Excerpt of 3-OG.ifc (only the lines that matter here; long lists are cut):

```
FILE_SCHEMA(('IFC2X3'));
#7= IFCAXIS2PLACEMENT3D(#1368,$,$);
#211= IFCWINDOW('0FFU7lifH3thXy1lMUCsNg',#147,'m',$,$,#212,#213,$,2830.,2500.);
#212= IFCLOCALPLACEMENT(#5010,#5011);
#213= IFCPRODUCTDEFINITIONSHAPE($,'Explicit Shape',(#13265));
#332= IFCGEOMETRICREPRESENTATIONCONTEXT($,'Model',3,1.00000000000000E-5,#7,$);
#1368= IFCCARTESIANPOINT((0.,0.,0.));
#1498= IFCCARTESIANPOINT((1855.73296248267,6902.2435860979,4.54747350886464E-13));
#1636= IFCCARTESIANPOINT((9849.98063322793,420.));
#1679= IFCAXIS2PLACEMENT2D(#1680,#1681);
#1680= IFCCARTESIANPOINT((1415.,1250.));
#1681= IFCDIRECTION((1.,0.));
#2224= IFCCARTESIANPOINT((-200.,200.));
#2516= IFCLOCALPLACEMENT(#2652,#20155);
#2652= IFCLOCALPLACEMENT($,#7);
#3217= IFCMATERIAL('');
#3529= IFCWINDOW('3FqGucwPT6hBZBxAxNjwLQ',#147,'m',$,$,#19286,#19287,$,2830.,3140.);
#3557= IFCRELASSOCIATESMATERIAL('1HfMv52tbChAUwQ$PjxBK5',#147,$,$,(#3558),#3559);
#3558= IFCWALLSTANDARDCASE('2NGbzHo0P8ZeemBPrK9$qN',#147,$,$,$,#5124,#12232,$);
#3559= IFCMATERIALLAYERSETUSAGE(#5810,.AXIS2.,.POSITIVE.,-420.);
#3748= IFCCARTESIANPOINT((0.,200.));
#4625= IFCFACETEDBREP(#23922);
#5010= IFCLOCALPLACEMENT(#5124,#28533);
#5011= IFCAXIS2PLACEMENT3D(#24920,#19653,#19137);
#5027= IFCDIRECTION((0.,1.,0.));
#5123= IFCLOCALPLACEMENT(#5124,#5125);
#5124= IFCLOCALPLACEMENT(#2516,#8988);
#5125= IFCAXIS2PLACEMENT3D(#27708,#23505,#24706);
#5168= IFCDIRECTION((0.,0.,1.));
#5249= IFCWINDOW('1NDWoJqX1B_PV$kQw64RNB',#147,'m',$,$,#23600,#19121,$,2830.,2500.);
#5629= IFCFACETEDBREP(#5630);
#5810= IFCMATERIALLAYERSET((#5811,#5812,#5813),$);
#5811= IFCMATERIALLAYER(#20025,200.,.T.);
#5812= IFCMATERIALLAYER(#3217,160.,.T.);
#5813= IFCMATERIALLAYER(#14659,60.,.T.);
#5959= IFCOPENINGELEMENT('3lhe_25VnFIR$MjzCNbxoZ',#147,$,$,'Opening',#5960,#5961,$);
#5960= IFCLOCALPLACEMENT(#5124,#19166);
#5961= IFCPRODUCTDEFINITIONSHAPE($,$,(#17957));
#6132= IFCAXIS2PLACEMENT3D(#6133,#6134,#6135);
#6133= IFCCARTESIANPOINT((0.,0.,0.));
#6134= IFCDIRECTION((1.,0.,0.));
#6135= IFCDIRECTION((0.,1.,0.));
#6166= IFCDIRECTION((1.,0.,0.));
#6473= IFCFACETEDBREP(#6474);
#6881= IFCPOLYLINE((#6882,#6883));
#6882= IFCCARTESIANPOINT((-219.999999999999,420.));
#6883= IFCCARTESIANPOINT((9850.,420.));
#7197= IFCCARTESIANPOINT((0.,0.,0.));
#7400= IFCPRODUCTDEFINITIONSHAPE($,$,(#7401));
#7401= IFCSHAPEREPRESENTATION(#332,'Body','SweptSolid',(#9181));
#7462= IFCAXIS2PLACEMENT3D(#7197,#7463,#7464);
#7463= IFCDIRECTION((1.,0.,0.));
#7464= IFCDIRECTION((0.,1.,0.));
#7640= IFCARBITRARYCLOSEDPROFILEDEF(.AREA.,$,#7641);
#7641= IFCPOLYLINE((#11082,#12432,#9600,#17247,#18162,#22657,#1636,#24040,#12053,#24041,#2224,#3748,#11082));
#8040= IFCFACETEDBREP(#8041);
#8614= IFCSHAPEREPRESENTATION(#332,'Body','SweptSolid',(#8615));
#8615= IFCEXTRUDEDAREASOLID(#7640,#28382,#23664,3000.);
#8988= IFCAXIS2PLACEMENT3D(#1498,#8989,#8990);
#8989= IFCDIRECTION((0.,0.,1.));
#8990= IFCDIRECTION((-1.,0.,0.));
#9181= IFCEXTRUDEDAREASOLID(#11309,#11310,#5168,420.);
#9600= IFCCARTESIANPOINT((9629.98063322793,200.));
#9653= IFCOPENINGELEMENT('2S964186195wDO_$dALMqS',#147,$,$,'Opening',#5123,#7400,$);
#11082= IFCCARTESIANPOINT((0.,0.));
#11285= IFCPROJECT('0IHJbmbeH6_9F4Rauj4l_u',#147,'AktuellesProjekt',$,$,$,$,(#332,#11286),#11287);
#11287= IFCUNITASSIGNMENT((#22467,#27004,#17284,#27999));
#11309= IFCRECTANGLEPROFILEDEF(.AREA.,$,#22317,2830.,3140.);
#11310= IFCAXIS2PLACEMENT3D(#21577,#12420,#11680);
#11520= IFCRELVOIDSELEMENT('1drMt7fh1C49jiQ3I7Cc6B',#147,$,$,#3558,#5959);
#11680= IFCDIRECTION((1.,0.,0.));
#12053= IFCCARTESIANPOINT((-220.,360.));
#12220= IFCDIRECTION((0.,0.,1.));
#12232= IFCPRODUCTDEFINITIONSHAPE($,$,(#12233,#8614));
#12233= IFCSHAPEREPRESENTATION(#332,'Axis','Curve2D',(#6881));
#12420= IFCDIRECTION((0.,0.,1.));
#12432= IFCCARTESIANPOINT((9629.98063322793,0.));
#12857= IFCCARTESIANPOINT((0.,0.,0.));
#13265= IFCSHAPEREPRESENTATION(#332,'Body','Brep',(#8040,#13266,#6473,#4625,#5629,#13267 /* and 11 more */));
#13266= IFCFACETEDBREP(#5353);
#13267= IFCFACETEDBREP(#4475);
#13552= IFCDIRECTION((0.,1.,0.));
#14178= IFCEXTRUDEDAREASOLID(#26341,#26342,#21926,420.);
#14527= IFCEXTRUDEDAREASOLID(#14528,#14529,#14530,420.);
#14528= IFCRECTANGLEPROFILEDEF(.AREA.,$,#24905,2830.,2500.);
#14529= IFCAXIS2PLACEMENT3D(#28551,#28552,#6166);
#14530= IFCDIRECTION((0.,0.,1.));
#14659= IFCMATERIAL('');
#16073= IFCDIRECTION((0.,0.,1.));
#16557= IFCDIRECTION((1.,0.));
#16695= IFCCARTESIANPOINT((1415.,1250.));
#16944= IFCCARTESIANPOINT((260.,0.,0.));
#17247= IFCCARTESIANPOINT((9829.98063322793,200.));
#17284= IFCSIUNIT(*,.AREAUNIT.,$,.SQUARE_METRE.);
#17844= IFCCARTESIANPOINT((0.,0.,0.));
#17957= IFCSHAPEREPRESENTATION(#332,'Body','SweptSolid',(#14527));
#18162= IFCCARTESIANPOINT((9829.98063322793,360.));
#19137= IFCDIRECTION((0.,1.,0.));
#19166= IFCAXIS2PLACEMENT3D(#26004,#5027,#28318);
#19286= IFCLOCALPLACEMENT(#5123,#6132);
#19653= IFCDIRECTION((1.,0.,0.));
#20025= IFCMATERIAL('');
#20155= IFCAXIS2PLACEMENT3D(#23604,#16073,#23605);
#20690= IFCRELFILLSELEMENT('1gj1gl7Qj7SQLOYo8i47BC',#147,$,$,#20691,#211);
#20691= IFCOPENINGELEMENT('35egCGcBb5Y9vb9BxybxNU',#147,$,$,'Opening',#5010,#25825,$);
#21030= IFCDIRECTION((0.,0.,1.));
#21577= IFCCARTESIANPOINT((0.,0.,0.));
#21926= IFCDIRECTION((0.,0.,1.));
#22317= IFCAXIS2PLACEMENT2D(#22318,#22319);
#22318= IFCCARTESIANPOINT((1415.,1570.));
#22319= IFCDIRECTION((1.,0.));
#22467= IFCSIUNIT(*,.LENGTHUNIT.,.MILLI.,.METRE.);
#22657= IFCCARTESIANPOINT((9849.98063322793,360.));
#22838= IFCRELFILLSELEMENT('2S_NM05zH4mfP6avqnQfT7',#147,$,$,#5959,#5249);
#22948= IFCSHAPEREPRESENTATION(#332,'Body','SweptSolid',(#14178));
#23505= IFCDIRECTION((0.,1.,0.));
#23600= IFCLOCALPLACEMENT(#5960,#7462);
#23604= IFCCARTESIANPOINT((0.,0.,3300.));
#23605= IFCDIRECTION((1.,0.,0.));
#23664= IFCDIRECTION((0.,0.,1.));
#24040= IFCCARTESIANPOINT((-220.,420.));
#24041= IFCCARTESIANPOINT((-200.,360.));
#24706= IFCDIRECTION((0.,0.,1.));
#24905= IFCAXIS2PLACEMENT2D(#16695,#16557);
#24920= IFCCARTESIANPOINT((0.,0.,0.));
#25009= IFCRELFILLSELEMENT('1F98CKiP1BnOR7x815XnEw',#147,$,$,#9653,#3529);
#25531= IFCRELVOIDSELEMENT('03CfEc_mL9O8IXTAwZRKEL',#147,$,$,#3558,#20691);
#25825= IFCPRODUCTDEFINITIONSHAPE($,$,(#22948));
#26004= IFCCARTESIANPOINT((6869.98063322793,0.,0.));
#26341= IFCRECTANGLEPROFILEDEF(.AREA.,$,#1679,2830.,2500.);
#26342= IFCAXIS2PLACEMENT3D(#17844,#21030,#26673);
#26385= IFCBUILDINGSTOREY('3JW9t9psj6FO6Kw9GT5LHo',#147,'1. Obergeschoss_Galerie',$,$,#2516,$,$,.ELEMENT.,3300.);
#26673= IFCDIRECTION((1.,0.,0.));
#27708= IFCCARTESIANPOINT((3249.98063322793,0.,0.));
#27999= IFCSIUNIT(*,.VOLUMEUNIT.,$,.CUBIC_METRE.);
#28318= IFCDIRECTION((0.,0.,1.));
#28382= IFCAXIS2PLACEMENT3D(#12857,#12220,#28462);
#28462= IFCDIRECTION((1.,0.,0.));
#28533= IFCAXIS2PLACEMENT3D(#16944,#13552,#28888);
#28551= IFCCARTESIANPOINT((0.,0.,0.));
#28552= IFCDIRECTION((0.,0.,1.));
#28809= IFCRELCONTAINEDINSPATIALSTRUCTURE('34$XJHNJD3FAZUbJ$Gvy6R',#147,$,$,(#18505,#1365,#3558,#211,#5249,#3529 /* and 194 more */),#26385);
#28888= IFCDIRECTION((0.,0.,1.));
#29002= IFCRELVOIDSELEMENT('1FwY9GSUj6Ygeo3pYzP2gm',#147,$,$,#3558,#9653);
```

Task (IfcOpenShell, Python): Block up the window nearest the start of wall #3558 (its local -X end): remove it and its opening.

```python
import ifcopenshell
import ifcopenshell.api.feature
import ifcopenshell.api.root
import ifcopenshell.geom
import ifcopenshell.util.shape

model = ifcopenshell.open("3-OG.ifc")
settings = ifcopenshell.geom.settings()


def volume(element):
    """Net volume in cubic metres, openings subtracted."""
    shape = ifcopenshell.geom.create_shape(settings, element)
    return ifcopenshell.util.shape.get_volume(shape.geometry)


window = model.by_guid("0FFU7lifH3thXy1lMUCsNg")
opening = window.FillsVoids[0].RelatingOpeningElement
wall = opening.VoidsElements[0].RelatingBuildingElement
before = volume(wall)

ifcopenshell.api.root.remove_product(model, product=window)
ifcopenshell.api.feature.remove_feature(model, feature=opening)

after = volume(wall)

print(f"wall volume {before:.3f} -> {after:.3f} m3")

model.write("3-OG_rev.ifc")
```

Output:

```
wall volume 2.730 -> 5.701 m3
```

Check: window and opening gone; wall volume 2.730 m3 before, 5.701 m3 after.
